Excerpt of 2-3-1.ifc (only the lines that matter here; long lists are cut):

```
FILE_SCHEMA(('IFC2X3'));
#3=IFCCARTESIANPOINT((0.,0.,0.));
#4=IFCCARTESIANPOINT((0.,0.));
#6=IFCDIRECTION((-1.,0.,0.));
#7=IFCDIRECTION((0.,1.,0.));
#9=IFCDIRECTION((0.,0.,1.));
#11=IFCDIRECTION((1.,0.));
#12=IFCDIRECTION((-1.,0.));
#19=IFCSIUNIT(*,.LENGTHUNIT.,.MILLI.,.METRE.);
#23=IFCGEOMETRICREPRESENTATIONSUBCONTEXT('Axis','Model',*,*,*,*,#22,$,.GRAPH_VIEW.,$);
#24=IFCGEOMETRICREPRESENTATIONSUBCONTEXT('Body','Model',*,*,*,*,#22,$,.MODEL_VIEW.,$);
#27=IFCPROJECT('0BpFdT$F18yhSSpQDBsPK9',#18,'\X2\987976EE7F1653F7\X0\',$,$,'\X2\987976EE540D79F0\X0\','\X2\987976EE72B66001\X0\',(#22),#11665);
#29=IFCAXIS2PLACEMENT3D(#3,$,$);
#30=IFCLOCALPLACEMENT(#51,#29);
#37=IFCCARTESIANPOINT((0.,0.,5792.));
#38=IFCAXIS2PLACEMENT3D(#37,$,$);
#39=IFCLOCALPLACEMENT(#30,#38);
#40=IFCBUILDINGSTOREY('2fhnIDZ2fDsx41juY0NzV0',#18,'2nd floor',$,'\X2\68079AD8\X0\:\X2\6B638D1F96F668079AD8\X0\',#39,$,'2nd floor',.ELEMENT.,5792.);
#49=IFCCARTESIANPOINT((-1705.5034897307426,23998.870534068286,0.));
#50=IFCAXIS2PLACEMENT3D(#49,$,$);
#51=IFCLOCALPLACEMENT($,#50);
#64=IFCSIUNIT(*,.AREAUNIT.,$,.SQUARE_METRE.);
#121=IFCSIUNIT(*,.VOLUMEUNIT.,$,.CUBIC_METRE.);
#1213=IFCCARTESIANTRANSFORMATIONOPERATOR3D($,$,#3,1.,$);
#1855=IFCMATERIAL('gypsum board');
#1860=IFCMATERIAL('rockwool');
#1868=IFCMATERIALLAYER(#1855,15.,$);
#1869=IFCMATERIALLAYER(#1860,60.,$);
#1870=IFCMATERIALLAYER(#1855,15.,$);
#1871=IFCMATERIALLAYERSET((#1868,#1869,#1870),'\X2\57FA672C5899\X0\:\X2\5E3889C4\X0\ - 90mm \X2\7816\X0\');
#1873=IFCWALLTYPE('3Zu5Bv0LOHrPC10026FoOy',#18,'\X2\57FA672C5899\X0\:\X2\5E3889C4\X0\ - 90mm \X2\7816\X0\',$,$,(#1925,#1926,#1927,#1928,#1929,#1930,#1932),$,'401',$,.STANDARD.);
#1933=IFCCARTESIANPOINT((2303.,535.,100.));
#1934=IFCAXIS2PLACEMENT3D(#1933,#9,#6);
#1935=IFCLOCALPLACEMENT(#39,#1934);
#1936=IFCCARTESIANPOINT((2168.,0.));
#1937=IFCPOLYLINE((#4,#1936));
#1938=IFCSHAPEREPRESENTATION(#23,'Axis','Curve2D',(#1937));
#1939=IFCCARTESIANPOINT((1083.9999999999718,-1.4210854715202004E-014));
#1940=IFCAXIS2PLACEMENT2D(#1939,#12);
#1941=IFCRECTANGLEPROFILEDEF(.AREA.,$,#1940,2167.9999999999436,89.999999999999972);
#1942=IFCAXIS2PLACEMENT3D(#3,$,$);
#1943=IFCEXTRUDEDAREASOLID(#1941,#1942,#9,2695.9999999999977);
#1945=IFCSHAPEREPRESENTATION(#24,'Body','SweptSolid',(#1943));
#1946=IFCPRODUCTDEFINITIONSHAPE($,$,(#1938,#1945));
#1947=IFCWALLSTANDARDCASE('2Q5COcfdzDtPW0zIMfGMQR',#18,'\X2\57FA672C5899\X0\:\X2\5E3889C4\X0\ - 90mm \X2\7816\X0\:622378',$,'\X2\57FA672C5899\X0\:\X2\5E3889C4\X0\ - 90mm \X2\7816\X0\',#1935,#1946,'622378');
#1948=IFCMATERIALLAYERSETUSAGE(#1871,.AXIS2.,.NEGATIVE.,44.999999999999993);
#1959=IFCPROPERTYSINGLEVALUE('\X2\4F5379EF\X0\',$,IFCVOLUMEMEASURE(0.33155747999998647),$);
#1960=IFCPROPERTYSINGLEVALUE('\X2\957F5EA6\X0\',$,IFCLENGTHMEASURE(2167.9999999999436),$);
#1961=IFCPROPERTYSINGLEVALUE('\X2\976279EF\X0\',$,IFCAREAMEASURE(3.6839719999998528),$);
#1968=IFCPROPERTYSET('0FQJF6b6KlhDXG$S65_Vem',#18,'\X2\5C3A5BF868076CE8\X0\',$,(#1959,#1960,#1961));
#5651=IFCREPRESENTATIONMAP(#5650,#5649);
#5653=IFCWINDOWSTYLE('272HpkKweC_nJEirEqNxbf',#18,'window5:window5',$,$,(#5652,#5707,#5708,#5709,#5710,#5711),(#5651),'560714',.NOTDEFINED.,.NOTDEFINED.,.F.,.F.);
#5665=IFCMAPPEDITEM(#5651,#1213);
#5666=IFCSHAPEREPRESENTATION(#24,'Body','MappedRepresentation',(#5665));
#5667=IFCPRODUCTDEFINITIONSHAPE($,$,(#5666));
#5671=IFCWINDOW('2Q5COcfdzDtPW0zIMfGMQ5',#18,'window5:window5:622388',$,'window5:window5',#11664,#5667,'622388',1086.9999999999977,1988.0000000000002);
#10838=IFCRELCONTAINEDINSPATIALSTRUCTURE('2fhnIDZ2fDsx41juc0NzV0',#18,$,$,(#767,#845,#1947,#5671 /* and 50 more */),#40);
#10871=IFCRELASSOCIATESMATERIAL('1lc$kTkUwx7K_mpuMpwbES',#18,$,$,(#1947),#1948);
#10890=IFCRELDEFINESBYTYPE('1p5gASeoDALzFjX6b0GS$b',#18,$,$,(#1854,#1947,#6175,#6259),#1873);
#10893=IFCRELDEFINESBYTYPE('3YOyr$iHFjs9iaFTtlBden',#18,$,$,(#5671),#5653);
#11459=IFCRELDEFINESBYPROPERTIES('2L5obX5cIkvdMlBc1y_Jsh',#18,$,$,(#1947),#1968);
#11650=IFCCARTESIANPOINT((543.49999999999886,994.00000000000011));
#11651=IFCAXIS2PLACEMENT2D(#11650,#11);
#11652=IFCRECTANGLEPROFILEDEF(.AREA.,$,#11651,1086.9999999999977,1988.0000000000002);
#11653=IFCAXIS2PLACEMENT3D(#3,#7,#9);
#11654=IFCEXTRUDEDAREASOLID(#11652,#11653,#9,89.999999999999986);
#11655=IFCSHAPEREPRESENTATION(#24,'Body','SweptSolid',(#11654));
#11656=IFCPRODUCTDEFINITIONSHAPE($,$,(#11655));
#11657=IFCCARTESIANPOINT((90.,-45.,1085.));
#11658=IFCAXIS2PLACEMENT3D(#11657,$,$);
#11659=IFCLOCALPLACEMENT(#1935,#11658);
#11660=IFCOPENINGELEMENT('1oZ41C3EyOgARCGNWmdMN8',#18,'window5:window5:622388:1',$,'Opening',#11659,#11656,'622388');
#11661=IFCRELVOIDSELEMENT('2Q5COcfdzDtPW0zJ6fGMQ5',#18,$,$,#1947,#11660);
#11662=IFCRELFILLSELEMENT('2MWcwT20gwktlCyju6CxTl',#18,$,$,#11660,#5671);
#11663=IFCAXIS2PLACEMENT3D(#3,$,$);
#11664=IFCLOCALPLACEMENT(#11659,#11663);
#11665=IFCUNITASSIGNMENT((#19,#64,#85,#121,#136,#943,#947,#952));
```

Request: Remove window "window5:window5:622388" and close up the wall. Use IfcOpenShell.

```python
import ifcopenshell
import ifcopenshell.api.feature
import ifcopenshell.api.pset
import ifcopenshell.api.root
import ifcopenshell.geom
import ifcopenshell.util.element
import ifcopenshell.util.shape
import ifcopenshell.util.unit

model = ifcopenshell.open("2-3-1.ifc")
area_scale = ifcopenshell.util.unit.calculate_unit_scale(model, "AREAUNIT")
volume_scale = ifcopenshell.util.unit.calculate_unit_scale(model, "VOLUMEUNIT")
settings = ifcopenshell.geom.settings()


def volume(element):
    """Net volume in cubic metres, openings subtracted."""
    shape = ifcopenshell.geom.create_shape(settings, element)
    return ifcopenshell.util.shape.get_volume(shape.geometry)


window = model.by_id(5671)
opening = window.FillsVoids[0].RelatingOpeningElement
wall = opening.VoidsElements[0].RelatingBuildingElement
before = volume(wall)

ifcopenshell.api.root.remove_product(model, product=window)
ifcopenshell.api.feature.remove_feature(model, feature=opening)

after = volume(wall)
thickness = 0.09  # wall thickness in metres

# Update the wall's stored quantities.
pset = model.by_id(ifcopenshell.util.element.get_pset(wall, "尺寸标注", should_inherit=False)["id"])
ifcopenshell.api.pset.edit_pset(model, pset=pset, properties={
    "体积": model.create_entity("IfcVolumeMeasure", after / volume_scale),
    "面积": model.create_entity("IfcAreaMeasure", after / thickness / area_scale),
})

print(f"wall volume {before:.3f} -> {after:.3f} m3")

model.write("2-3-1-out.ifc")
```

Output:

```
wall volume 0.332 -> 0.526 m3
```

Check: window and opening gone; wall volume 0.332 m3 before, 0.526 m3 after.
